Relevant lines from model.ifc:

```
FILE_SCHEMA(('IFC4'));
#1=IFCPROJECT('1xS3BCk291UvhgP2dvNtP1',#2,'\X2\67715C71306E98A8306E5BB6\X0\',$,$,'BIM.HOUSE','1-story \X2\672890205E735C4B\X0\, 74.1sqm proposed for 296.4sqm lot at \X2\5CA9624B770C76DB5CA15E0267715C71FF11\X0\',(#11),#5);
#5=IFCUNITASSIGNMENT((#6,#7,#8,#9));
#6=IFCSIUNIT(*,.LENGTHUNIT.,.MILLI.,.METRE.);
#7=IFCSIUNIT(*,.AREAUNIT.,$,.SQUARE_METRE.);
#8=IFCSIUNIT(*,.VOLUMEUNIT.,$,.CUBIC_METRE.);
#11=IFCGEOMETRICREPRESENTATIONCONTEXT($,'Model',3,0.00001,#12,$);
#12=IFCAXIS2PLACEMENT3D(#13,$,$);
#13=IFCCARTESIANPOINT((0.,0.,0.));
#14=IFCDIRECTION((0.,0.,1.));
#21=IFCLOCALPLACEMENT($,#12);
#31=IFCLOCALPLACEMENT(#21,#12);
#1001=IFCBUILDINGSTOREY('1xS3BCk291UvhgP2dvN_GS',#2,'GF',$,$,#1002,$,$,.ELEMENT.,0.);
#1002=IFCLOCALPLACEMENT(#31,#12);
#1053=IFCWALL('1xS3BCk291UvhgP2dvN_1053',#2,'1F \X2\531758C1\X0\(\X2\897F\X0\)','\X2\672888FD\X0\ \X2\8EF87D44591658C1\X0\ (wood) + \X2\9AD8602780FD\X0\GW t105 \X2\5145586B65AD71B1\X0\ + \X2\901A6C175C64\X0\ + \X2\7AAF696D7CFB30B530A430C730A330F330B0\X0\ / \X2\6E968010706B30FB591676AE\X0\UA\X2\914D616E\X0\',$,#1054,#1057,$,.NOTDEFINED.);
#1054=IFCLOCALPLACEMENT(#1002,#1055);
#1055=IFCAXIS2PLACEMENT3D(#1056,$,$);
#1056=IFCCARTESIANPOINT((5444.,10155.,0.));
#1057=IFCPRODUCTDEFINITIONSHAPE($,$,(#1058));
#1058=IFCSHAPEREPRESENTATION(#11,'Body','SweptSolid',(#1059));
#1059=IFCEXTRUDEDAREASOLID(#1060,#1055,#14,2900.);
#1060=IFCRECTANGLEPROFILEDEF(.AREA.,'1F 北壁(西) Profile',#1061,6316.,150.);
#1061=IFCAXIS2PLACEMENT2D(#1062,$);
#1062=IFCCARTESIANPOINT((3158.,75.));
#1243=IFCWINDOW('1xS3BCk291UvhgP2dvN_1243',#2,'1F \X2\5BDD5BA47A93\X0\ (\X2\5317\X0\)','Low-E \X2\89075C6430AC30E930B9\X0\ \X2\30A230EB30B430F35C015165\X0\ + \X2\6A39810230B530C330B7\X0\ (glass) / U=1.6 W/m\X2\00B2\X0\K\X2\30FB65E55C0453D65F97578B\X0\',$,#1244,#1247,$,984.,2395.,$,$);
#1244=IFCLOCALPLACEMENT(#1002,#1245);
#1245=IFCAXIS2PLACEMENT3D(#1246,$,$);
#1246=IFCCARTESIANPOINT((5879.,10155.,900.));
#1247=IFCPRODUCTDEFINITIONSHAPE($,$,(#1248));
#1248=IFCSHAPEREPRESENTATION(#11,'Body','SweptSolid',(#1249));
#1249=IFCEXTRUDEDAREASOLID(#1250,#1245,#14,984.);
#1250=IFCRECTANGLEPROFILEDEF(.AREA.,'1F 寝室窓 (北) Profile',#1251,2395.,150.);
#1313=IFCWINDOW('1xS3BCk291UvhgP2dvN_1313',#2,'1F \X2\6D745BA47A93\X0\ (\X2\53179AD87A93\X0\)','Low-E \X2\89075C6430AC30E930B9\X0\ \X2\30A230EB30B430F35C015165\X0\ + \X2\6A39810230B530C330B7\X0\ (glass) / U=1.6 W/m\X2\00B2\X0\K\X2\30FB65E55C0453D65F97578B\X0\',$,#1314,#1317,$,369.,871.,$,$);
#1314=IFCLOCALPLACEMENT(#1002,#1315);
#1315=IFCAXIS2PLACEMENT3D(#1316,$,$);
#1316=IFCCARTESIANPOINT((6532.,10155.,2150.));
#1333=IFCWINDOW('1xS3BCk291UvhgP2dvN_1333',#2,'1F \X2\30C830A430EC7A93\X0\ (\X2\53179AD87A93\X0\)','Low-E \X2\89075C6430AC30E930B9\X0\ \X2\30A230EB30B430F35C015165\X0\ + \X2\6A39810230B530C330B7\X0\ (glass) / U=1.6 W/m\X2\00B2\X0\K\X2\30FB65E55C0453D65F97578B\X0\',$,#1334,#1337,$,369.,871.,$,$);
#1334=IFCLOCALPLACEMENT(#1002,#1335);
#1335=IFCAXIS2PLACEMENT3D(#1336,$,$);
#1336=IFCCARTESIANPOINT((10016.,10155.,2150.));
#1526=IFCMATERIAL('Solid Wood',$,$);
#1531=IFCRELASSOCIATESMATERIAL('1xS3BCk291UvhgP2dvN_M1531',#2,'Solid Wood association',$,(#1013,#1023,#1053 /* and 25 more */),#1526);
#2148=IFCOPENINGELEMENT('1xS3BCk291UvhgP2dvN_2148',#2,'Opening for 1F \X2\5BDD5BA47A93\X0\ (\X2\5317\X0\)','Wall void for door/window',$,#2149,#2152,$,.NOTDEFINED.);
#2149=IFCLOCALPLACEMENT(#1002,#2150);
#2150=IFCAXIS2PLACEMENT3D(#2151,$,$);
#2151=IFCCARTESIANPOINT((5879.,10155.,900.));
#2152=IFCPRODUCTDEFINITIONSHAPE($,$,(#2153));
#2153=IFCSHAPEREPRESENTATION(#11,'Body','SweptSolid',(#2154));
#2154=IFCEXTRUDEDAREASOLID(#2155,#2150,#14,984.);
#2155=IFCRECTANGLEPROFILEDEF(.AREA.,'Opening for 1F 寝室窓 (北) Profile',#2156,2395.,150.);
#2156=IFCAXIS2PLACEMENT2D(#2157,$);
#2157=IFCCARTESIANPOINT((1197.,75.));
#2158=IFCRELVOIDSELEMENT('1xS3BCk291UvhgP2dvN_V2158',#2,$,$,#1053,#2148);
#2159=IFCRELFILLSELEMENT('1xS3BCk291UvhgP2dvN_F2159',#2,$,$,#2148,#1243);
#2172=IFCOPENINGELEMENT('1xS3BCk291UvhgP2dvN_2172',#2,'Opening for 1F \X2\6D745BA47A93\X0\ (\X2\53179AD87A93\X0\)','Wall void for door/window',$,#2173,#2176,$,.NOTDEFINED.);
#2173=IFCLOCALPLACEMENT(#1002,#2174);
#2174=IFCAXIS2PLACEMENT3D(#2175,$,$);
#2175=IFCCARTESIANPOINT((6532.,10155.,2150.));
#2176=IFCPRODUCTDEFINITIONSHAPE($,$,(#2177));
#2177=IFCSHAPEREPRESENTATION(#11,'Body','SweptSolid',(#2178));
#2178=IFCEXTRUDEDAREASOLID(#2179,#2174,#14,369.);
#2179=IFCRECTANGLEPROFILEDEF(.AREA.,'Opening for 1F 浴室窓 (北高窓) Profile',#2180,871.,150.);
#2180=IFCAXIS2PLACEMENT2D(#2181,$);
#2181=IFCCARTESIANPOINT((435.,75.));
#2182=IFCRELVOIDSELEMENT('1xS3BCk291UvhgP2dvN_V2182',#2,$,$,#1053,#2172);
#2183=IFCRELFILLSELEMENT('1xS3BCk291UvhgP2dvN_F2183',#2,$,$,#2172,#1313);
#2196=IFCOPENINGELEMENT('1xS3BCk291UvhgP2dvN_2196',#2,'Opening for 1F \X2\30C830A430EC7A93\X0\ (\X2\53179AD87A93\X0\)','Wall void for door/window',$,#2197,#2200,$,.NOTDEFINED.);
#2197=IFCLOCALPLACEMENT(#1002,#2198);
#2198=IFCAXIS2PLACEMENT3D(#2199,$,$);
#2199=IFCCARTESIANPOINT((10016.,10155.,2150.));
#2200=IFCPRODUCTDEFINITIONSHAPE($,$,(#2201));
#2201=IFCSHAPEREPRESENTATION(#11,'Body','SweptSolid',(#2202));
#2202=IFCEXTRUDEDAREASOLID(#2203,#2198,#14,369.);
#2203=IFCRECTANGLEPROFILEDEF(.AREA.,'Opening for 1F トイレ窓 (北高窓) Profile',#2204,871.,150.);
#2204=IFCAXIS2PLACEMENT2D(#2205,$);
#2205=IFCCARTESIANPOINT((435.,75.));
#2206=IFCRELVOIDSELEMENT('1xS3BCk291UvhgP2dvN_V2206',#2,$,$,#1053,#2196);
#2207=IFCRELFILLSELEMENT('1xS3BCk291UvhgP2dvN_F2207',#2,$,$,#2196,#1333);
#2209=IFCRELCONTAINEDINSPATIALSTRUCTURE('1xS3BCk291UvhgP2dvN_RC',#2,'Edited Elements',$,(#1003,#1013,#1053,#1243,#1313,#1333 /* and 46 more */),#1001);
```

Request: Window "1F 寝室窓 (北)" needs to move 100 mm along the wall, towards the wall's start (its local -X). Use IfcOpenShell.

```python
import ifcopenshell
import ifcopenshell.api.geometry
import ifcopenshell.util.placement
import ifcopenshell.util.unit

model = ifcopenshell.open("model.ifc")
unit_scale = ifcopenshell.util.unit.calculate_unit_scale(model)

window = model.by_guid("1xS3BCk291UvhgP2dvN_1243")
opening = window.FillsVoids[0].RelatingOpeningElement
wall = opening.VoidsElements[0].RelatingBuildingElement

wall_matrix = ifcopenshell.util.placement.get_local_placement(wall.ObjectPlacement)
shift = wall_matrix[:3, 0] * -0.1 / unit_scale
before = ifcopenshell.util.placement.get_local_placement(window.ObjectPlacement)[:3, 3].copy()

# The window is not placed relative to its opening, so move both.
for product in (opening, window):
    matrix = ifcopenshell.util.placement.get_local_placement(product.ObjectPlacement)
    matrix[:3, 3] += shift
    ifcopenshell.api.geometry.edit_object_placement(model, product=product, matrix=matrix, is_si=False)

after = ifcopenshell.util.placement.get_local_placement(window.ObjectPlacement)[:3, 3]
print("window moved by", (after - before).round(3) + 0.0)

model.write("model_edited.ifc")
```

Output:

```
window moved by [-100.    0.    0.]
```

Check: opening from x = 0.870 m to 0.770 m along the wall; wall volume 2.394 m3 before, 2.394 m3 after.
